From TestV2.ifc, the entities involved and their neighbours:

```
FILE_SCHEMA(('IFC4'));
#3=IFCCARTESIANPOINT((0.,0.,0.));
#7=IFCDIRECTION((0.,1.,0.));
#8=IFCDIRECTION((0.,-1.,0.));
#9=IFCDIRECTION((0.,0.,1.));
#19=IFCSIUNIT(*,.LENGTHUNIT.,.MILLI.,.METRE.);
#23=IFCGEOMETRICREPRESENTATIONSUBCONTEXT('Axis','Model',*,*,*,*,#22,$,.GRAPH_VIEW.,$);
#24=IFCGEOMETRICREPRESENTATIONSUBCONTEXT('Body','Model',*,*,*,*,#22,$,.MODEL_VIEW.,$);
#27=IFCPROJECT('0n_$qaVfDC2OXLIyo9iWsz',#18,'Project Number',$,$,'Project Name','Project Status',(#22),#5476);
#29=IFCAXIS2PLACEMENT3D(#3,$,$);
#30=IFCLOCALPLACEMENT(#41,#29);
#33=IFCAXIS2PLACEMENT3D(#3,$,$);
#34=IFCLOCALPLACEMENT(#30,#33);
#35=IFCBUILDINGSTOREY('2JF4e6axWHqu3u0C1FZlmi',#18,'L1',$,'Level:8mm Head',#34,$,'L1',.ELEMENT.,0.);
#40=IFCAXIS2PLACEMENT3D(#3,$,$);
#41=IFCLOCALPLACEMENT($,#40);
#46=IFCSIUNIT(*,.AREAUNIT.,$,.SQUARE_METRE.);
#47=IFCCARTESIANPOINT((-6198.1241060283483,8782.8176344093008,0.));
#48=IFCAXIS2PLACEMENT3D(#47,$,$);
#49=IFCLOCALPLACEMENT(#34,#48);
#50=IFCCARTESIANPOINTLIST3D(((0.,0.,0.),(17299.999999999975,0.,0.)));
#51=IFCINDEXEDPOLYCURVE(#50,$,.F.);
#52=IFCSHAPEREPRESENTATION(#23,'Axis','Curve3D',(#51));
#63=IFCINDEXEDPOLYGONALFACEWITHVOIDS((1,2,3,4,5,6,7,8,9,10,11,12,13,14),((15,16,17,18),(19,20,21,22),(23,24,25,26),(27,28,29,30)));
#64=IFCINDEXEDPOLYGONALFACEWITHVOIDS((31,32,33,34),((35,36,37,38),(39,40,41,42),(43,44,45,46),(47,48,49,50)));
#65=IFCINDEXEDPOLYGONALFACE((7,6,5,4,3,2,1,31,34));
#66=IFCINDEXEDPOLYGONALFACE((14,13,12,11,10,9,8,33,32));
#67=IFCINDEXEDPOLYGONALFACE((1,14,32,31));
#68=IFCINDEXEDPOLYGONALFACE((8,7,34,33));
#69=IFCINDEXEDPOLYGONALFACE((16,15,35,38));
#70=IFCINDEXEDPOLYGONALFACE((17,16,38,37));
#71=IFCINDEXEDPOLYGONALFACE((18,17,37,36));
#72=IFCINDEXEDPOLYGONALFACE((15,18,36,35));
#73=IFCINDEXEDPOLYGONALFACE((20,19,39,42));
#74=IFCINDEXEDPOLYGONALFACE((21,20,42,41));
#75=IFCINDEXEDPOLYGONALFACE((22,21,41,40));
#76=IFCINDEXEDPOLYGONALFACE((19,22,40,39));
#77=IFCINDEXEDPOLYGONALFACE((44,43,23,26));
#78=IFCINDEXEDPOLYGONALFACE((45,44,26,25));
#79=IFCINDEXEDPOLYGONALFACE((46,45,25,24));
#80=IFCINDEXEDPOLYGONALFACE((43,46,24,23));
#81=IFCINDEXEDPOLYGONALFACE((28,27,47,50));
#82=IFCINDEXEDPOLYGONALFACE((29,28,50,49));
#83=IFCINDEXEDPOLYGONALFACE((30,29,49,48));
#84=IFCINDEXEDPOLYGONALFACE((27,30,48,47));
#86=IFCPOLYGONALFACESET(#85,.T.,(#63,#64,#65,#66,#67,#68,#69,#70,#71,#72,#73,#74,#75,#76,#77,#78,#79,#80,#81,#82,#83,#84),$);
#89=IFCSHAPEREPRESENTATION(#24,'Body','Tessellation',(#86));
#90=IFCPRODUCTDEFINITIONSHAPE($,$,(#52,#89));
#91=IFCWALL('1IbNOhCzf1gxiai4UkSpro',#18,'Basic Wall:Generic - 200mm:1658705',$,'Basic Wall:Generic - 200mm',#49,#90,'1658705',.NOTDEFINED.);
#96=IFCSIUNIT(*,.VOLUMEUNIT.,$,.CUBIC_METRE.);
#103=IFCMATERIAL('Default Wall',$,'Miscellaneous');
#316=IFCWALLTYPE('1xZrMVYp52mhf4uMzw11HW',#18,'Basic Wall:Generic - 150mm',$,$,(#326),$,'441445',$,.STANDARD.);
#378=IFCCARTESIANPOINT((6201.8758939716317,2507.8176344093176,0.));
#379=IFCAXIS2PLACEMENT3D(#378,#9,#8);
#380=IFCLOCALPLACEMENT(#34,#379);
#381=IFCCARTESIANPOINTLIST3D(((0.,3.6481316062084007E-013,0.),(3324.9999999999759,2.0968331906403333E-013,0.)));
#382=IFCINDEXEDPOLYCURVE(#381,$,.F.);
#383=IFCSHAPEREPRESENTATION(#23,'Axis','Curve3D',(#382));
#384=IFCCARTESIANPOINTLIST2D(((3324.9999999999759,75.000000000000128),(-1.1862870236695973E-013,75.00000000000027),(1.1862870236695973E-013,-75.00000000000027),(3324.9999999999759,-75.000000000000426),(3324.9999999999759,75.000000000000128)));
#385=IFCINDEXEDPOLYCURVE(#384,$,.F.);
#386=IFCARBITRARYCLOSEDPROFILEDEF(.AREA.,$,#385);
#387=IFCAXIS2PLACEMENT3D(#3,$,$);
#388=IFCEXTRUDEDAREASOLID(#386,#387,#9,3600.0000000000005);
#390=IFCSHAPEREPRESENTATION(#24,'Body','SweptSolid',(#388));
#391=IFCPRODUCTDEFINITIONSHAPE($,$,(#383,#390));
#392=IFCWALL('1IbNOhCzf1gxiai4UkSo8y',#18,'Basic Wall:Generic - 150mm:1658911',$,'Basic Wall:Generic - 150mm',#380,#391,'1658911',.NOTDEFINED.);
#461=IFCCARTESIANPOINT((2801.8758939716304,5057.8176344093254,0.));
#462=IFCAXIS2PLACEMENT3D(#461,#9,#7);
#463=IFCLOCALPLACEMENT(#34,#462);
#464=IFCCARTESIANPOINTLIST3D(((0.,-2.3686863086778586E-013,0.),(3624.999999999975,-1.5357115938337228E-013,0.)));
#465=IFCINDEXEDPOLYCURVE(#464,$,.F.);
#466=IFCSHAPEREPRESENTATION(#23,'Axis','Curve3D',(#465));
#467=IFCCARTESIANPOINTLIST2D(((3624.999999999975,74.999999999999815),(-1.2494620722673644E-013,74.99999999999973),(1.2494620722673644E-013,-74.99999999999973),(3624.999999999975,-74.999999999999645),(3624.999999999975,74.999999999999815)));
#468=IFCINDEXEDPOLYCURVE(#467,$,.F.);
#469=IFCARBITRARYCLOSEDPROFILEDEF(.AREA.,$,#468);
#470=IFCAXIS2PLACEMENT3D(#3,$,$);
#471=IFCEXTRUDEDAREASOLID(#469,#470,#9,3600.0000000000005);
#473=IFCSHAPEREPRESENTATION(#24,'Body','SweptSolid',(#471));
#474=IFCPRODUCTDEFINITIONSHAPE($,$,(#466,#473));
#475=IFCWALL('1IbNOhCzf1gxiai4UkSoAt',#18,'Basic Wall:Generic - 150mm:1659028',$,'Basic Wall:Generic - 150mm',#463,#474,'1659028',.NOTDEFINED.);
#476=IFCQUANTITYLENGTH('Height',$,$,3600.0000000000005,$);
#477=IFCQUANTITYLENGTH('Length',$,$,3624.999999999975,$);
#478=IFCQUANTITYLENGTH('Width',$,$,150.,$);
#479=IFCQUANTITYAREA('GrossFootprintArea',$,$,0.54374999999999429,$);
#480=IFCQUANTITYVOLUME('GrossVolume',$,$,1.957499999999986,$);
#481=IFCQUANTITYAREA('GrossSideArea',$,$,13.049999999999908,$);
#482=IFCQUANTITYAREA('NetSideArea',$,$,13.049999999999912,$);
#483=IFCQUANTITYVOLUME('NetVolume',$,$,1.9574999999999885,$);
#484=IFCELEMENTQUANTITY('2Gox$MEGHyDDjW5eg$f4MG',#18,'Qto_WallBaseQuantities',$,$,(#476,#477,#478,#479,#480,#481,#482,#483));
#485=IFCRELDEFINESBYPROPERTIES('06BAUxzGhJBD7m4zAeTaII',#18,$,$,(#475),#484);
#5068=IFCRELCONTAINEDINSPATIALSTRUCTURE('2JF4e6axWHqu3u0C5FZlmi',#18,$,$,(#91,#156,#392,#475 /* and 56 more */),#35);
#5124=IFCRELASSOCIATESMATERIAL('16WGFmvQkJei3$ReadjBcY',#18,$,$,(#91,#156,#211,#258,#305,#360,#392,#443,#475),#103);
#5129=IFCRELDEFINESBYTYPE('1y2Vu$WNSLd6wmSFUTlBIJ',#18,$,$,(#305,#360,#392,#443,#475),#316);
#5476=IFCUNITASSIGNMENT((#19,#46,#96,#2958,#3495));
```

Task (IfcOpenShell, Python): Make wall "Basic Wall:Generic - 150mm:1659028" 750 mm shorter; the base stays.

```python
import ifcopenshell
import ifcopenshell.api.pset
import ifcopenshell.geom
import ifcopenshell.util.element
import ifcopenshell.util.representation
import ifcopenshell.util.shape
import ifcopenshell.util.unit

model = ifcopenshell.open("TestV2.ifc")
unit_scale = ifcopenshell.util.unit.calculate_unit_scale(model)
area_scale = ifcopenshell.util.unit.calculate_unit_scale(model, "AREAUNIT")
volume_scale = ifcopenshell.util.unit.calculate_unit_scale(model, "VOLUMEUNIT")
settings = ifcopenshell.geom.settings()


def volume(element):
    """Net volume in cubic metres, openings subtracted."""
    shape = ifcopenshell.geom.create_shape(settings, element)
    return ifcopenshell.util.shape.get_volume(shape.geometry)


wall = model.by_guid("1IbNOhCzf1gxiai4UkSoAt")
before = volume(wall)

body = ifcopenshell.util.representation.get_representation(wall, "Model", "Body")
solid = body.Items[0]
old_height = solid.Depth
solid.Depth -= 750.0
after = volume(wall)
thickness = 0.15  # wall thickness in metres

# Update the stored height, areas and volumes.
qto = model.by_id(ifcopenshell.util.element.get_pset(wall, "Qto_WallBaseQuantities", should_inherit=False)["id"])
ifcopenshell.api.pset.edit_qto(model, qto=qto, properties={
    "Height": solid.Depth,
    "GrossVolume": ifcopenshell.util.element.get_pset(wall, "Qto_WallBaseQuantities", "GrossVolume") * solid.Depth / old_height,
    "GrossSideArea": ifcopenshell.util.element.get_pset(wall, "Qto_WallBaseQuantities", "GrossSideArea") * solid.Depth / old_height,
    "NetSideArea": after / thickness / area_scale,
    "NetVolume": after / volume_scale,
})

print(f"height {old_height:g} -> {solid.Depth:g}, volume {before:.3f} -> {after:.3f} m3")

model.write("TestV2_v2.ifc")
```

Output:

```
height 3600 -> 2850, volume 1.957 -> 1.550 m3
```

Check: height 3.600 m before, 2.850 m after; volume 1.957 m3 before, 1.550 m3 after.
